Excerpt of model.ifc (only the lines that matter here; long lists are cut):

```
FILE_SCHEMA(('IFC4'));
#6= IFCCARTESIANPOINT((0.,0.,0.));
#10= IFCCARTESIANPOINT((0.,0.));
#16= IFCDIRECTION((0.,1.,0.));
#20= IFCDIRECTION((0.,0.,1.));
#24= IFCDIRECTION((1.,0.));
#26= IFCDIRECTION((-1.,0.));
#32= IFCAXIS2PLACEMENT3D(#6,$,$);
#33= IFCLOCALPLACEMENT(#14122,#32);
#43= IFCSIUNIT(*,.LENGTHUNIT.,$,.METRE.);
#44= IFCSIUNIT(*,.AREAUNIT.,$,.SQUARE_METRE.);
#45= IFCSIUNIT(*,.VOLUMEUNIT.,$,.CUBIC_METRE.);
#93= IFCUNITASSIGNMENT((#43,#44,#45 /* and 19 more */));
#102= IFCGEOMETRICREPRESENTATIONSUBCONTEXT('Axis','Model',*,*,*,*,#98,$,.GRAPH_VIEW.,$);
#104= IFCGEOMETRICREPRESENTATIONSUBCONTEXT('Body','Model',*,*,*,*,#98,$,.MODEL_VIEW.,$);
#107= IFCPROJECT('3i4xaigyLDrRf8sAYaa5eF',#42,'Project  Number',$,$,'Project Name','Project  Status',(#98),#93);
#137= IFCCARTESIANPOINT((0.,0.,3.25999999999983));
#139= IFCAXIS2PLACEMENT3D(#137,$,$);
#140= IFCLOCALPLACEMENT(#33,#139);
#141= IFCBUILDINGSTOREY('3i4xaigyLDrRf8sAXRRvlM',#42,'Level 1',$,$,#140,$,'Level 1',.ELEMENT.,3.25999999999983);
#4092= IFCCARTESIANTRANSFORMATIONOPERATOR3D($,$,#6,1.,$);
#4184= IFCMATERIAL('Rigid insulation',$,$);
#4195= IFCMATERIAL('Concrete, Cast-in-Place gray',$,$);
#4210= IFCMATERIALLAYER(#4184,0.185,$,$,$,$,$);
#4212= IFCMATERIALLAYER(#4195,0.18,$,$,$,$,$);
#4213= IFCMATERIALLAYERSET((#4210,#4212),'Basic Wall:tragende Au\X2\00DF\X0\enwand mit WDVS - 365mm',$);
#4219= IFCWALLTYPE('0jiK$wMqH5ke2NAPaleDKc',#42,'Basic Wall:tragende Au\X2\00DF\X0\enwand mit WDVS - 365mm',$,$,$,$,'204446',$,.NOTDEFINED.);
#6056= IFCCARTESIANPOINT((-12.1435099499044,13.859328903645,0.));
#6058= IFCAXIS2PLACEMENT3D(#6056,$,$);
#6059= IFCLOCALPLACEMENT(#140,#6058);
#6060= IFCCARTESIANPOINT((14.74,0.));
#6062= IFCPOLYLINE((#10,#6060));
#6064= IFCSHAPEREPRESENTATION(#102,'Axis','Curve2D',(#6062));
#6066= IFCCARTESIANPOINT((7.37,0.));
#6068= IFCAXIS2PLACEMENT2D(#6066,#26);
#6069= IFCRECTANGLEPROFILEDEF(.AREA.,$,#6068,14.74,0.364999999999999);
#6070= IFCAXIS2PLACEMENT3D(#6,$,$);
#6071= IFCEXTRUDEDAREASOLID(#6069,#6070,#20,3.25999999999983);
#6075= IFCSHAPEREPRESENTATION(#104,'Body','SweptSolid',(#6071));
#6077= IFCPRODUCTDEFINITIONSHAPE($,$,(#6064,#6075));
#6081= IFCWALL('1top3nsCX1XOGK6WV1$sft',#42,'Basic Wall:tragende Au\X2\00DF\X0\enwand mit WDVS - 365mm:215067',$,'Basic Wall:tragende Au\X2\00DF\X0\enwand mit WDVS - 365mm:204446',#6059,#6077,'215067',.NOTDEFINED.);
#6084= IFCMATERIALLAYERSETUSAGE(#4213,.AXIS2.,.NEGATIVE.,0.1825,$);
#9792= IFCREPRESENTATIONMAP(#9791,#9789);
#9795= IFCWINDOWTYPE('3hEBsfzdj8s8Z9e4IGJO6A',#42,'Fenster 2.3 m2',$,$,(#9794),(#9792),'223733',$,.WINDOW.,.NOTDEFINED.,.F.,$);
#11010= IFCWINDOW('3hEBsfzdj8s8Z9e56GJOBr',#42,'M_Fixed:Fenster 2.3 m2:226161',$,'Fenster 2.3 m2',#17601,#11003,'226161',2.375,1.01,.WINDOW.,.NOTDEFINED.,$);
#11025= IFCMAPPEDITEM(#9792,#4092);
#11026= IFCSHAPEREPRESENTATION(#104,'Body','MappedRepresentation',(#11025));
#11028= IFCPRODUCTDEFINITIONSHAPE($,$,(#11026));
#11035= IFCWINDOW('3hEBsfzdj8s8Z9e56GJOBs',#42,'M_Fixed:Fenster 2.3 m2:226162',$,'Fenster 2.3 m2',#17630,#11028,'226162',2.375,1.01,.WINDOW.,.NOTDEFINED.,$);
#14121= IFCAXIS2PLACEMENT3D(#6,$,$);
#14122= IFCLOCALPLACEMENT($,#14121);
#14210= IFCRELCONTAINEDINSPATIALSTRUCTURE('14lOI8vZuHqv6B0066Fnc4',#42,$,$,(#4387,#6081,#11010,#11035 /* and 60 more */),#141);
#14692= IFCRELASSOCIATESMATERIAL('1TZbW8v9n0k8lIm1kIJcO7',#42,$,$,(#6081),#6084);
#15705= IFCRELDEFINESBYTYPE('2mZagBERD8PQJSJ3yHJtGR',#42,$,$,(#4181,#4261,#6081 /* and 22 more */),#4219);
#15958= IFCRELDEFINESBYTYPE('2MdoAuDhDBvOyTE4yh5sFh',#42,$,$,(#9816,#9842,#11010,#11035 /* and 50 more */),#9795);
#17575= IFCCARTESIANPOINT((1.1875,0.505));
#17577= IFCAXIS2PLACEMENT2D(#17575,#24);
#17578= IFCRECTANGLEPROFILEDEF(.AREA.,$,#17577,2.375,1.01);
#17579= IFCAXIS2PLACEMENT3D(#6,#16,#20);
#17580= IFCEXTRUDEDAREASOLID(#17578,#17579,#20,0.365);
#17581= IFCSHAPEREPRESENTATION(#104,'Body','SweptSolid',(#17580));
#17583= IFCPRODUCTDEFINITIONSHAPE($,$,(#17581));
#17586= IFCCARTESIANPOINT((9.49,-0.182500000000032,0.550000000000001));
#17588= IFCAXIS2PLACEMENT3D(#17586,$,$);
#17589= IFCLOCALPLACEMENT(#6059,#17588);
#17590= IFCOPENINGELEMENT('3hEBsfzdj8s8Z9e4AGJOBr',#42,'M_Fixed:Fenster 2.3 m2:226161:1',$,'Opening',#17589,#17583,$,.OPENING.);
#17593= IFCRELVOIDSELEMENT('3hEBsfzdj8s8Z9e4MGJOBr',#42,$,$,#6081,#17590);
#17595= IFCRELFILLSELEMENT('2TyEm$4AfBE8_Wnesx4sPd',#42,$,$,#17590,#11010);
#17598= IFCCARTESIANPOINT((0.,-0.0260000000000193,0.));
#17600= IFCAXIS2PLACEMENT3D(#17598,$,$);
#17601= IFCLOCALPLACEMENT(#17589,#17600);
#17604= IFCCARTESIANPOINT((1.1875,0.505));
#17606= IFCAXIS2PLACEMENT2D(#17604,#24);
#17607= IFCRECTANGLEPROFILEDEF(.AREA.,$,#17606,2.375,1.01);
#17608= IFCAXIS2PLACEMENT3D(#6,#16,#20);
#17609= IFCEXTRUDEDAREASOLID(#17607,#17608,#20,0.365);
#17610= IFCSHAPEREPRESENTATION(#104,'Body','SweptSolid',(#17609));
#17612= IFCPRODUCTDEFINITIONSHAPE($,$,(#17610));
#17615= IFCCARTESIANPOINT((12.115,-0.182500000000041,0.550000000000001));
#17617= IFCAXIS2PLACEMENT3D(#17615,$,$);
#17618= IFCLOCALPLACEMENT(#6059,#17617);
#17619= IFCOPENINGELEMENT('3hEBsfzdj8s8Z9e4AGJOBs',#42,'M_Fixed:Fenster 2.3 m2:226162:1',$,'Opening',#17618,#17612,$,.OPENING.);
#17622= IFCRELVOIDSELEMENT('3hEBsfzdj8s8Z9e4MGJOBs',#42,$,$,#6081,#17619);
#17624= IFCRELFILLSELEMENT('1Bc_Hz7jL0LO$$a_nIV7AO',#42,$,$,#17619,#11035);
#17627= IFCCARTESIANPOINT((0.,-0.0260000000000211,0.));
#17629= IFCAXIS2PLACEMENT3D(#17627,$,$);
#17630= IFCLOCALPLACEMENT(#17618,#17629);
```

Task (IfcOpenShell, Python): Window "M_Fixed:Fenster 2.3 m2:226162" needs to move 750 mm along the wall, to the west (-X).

```python
import ifcopenshell
import ifcopenshell.api.geometry
import ifcopenshell.util.placement

model = ifcopenshell.open("model.ifc")

window = model.by_guid("3hEBsfzdj8s8Z9e56GJOBs")
opening = window.FillsVoids[0].RelatingOpeningElement
wall = opening.VoidsElements[0].RelatingBuildingElement

wall_matrix = ifcopenshell.util.placement.get_local_placement(wall.ObjectPlacement)
shift = wall_matrix[:3, 0] * -0.75
before = ifcopenshell.util.placement.get_local_placement(window.ObjectPlacement)[:3, 3].copy()

# The window is placed relative to its opening, so it follows when the opening moves.
matrix = ifcopenshell.util.placement.get_local_placement(opening.ObjectPlacement)
matrix[:3, 3] += shift
ifcopenshell.api.geometry.edit_object_placement(
    model, product=opening, matrix=matrix, is_si=False, should_transform_children=True
)

after = ifcopenshell.util.placement.get_local_placement(window.ObjectPlacement)[:3, 3]
print("window moved by", (after - before).round(3) + 0.0)

model.write("model-out.ifc")
```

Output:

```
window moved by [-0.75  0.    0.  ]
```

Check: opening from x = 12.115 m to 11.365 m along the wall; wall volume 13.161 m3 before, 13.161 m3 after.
